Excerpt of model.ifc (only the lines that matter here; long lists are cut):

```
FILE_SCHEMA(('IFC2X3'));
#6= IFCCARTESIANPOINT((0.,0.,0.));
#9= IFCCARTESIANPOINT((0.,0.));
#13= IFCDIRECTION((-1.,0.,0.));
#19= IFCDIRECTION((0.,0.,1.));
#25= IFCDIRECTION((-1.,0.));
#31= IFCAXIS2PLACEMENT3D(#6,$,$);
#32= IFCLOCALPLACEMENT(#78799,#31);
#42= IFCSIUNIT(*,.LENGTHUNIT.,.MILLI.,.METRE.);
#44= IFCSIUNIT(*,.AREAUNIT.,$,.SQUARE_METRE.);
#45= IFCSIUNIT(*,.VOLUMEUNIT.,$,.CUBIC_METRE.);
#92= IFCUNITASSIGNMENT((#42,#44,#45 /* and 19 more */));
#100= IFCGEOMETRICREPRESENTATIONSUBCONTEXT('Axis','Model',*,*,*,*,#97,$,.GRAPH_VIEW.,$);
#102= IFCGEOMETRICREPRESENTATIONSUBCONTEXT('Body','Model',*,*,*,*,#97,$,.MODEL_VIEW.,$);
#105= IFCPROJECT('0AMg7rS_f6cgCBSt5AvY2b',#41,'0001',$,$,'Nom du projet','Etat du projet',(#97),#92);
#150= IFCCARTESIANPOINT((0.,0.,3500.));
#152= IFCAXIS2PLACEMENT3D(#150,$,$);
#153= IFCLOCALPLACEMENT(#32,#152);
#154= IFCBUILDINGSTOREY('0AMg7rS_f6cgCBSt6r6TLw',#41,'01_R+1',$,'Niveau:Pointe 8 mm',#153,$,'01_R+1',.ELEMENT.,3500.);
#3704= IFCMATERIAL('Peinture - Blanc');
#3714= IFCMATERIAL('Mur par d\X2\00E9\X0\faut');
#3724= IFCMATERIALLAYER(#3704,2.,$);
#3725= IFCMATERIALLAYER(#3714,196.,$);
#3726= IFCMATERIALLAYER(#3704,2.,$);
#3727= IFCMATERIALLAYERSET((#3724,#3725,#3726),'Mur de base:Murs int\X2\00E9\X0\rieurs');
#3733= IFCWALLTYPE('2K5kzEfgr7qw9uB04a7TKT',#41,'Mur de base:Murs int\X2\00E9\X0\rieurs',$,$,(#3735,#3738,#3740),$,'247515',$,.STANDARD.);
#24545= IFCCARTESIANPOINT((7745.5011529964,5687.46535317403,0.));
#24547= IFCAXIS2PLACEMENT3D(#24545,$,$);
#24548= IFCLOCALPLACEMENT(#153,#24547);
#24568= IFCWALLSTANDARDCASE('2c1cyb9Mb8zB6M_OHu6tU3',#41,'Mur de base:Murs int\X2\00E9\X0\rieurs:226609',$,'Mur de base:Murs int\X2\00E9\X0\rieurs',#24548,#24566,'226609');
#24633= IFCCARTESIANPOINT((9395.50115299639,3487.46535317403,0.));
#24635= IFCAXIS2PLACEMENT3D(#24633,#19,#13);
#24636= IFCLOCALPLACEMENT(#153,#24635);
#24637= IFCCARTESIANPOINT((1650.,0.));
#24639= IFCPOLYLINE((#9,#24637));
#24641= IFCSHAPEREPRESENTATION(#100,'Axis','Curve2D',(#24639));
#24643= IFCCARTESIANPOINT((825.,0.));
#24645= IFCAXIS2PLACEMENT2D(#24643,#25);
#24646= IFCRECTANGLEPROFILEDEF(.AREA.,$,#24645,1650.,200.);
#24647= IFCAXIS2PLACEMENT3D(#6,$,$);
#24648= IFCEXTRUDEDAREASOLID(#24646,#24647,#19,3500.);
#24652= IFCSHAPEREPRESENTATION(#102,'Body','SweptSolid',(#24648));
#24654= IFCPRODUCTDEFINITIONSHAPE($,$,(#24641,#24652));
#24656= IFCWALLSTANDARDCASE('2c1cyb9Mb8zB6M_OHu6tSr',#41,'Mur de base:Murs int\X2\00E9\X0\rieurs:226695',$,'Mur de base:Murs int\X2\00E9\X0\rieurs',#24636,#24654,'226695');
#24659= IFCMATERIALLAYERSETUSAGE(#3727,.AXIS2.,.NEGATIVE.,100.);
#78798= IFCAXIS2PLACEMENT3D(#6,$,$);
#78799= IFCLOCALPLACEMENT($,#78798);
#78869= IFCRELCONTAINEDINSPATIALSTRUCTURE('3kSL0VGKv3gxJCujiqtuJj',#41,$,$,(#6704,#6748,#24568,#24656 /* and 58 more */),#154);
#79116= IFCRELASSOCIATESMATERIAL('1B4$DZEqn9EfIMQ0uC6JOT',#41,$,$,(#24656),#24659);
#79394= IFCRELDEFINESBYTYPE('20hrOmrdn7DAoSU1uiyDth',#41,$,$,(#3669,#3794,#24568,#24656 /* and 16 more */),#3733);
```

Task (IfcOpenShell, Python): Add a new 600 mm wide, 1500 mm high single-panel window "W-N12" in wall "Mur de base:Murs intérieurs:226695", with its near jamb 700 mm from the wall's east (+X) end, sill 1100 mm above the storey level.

```python
import numpy as np
import ifcopenshell
import ifcopenshell.api.feature
import ifcopenshell.api.geometry
import ifcopenshell.api.root
import ifcopenshell.api.spatial
import ifcopenshell.api.type
import ifcopenshell.geom
import ifcopenshell.util.element
import ifcopenshell.util.placement
import ifcopenshell.util.representation
import ifcopenshell.util.shape
import ifcopenshell.util.unit

model = ifcopenshell.open("model.ifc")
unit_scale = ifcopenshell.util.unit.calculate_unit_scale(model)
settings = ifcopenshell.geom.settings()


def volume(element):
    """Net volume in cubic metres, openings subtracted."""
    shape = ifcopenshell.geom.create_shape(settings, element)
    return ifcopenshell.util.shape.get_volume(shape.geometry)


wall = model.by_guid("2c1cyb9Mb8zB6M_OHu6tSr")
storey = ifcopenshell.util.element.get_container(wall, ifc_class="IfcBuildingStorey")
context = ifcopenshell.util.representation.get_context(model, "Model", "Body", "MODEL_VIEW")
before = volume(wall)

width, height, from_end, sill = 0.6, 1.5, 0.7, 1.1  # metres

# The wall runs along its own X axis, and the end named is its -X end.
wall_shape = ifcopenshell.geom.create_shape(settings, wall)
x, y, z = ifcopenshell.util.shape.get_vertices(wall_shape.geometry).T
start = x.min() + from_end
face, thickness = float(y.min()), float(y.max() - y.min())
wall_matrix = ifcopenshell.util.placement.get_local_placement(wall.ObjectPlacement)
level = ifcopenshell.util.placement.get_local_placement(storey.ObjectPlacement)[2, 3]


def in_wall(x, y):
    """Placement at x, y metres in the wall's axes, at sill height."""
    matrix = wall_matrix.copy()
    matrix[:, 3] = wall_matrix @ np.array([x / unit_scale, y / unit_scale, 0.0, 1.0])
    matrix[2, 3] = level + sill / unit_scale
    return matrix


# Opening: a box that overshoots both wall faces by 50 mm.
opening = ifcopenshell.api.root.create_entity(model, ifc_class="IfcOpeningElement")
box = ifcopenshell.api.geometry.add_wall_representation(
    model, context=context, length=width, height=height, thickness=thickness + 0.1
)
ifcopenshell.api.geometry.assign_representation(model, product=opening, representation=box)
ifcopenshell.api.geometry.edit_object_placement(model, product=opening, matrix=in_wall(start, face - 0.05), is_si=False)
ifcopenshell.api.feature.add_feature(model, feature=opening, element=wall)

window = ifcopenshell.api.root.create_entity(model, ifc_class="IfcWindow", name="W-N12")
window.OverallWidth, window.OverallHeight = width / unit_scale, height / unit_scale
body = ifcopenshell.api.geometry.add_window_representation(
    model,
    context=context,
    overall_width=window.OverallWidth,
    overall_height=window.OverallHeight,
    partition_type="SINGLE_PANEL",
)
ifcopenshell.api.geometry.assign_representation(model, product=window, representation=body)
ifcopenshell.api.spatial.assign_container(model, products=[window], relating_structure=storey)
fills = ifcopenshell.api.feature.add_filling(model, opening=opening, element=window)
fills.OwnerHistory = window.OwnerHistory  # required in IFC2X3

# IFC2X3 keeps the operation on the window style.
style = ifcopenshell.api.root.create_entity(model, ifc_class="IfcWindowStyle", name="W-N12")
style.OperationType, style.ConstructionType = "SINGLE_PANEL", "NOTDEFINED"
style.ParameterTakesPrecedence = style.Sizeable = False
ifcopenshell.api.type.assign_type(model, related_objects=[window], relating_type=style)

# Centre the window in the wall's thickness.
ifcopenshell.api.geometry.edit_object_placement(model, product=window, matrix=in_wall(start, face), is_si=False)
window_shape = ifcopenshell.geom.create_shape(settings, window)
depth = ifcopenshell.util.shape.get_vertices(window_shape.geometry)[:, 1]
offset = face + thickness / 2 - (depth.min() + depth.max()) / 2
ifcopenshell.api.geometry.edit_object_placement(model, product=window, matrix=in_wall(start, offset), is_si=False)

after = volume(wall)

print(f"wall volume {before:.3f} -> {after:.3f} m3")

model.write("model_updated.ifc")
```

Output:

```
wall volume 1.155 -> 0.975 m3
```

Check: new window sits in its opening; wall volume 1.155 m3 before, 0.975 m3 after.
